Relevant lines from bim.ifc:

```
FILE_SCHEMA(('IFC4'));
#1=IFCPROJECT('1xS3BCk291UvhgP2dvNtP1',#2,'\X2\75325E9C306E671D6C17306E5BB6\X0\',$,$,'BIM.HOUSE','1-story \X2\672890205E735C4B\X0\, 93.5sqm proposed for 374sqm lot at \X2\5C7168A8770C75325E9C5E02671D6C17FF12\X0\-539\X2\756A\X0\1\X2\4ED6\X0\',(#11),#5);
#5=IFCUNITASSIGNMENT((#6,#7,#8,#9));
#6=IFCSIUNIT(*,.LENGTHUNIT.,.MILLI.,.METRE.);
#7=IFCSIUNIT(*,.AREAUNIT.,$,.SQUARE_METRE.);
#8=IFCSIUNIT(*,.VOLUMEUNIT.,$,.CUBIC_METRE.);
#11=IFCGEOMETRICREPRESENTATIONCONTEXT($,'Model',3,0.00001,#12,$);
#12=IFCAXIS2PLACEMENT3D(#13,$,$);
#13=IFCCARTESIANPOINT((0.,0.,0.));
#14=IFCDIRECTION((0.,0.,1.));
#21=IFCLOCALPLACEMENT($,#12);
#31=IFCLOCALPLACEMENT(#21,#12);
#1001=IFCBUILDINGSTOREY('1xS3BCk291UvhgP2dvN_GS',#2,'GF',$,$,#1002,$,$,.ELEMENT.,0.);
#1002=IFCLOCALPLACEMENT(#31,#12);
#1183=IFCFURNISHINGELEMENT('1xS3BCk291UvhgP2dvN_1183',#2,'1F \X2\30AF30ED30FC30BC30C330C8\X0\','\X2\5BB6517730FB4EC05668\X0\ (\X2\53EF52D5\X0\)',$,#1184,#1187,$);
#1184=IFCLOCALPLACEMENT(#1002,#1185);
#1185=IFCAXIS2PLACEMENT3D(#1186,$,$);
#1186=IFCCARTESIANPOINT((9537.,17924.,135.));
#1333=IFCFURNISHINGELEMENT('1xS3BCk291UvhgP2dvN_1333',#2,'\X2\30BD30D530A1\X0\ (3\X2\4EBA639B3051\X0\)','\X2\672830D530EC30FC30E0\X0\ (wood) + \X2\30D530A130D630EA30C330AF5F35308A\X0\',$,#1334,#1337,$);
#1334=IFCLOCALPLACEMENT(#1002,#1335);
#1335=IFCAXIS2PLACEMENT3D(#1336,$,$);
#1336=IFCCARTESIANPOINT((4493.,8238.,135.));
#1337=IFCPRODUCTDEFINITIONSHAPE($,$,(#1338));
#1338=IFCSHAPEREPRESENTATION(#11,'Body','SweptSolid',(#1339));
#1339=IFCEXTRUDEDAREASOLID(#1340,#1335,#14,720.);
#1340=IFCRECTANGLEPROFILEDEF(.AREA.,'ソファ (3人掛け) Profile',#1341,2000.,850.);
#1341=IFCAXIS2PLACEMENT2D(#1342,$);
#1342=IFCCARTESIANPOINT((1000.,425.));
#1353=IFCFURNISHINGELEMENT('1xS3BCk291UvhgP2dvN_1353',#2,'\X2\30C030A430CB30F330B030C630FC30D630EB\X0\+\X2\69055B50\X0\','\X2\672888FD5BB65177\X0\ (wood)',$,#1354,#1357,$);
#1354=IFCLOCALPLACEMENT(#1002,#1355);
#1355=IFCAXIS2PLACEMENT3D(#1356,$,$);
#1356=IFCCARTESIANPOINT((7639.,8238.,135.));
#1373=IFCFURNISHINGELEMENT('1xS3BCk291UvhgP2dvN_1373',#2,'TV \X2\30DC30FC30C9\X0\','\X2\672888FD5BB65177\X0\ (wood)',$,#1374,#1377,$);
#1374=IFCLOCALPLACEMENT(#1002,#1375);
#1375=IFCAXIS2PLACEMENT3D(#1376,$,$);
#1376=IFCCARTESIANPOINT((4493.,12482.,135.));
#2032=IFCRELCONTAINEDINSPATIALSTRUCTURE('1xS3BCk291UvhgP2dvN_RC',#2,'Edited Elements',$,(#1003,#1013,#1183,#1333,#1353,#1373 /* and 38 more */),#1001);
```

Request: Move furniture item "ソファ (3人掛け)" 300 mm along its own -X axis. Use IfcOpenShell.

```python
import ifcopenshell
import ifcopenshell.api.geometry
import ifcopenshell.util.placement
import ifcopenshell.util.unit

model = ifcopenshell.open("bim.ifc")
unit_scale = ifcopenshell.util.unit.calculate_unit_scale(model)

item = model.by_guid("1xS3BCk291UvhgP2dvN_1333")
matrix = ifcopenshell.util.placement.get_local_placement(item.ObjectPlacement)
matrix[:3, 3] -= matrix[:3, 0] * 0.3 / unit_scale
ifcopenshell.api.geometry.edit_object_placement(model, product=item, matrix=matrix, is_si=False)

print(ifcopenshell.util.placement.get_local_placement(item.ObjectPlacement).round(3) + 0.0)

model.write("bim_v2.ifc")
```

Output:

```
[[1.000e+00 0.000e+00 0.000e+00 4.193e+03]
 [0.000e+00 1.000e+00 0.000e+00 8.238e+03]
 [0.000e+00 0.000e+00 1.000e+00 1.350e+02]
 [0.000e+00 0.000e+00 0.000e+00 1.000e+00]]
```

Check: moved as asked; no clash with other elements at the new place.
